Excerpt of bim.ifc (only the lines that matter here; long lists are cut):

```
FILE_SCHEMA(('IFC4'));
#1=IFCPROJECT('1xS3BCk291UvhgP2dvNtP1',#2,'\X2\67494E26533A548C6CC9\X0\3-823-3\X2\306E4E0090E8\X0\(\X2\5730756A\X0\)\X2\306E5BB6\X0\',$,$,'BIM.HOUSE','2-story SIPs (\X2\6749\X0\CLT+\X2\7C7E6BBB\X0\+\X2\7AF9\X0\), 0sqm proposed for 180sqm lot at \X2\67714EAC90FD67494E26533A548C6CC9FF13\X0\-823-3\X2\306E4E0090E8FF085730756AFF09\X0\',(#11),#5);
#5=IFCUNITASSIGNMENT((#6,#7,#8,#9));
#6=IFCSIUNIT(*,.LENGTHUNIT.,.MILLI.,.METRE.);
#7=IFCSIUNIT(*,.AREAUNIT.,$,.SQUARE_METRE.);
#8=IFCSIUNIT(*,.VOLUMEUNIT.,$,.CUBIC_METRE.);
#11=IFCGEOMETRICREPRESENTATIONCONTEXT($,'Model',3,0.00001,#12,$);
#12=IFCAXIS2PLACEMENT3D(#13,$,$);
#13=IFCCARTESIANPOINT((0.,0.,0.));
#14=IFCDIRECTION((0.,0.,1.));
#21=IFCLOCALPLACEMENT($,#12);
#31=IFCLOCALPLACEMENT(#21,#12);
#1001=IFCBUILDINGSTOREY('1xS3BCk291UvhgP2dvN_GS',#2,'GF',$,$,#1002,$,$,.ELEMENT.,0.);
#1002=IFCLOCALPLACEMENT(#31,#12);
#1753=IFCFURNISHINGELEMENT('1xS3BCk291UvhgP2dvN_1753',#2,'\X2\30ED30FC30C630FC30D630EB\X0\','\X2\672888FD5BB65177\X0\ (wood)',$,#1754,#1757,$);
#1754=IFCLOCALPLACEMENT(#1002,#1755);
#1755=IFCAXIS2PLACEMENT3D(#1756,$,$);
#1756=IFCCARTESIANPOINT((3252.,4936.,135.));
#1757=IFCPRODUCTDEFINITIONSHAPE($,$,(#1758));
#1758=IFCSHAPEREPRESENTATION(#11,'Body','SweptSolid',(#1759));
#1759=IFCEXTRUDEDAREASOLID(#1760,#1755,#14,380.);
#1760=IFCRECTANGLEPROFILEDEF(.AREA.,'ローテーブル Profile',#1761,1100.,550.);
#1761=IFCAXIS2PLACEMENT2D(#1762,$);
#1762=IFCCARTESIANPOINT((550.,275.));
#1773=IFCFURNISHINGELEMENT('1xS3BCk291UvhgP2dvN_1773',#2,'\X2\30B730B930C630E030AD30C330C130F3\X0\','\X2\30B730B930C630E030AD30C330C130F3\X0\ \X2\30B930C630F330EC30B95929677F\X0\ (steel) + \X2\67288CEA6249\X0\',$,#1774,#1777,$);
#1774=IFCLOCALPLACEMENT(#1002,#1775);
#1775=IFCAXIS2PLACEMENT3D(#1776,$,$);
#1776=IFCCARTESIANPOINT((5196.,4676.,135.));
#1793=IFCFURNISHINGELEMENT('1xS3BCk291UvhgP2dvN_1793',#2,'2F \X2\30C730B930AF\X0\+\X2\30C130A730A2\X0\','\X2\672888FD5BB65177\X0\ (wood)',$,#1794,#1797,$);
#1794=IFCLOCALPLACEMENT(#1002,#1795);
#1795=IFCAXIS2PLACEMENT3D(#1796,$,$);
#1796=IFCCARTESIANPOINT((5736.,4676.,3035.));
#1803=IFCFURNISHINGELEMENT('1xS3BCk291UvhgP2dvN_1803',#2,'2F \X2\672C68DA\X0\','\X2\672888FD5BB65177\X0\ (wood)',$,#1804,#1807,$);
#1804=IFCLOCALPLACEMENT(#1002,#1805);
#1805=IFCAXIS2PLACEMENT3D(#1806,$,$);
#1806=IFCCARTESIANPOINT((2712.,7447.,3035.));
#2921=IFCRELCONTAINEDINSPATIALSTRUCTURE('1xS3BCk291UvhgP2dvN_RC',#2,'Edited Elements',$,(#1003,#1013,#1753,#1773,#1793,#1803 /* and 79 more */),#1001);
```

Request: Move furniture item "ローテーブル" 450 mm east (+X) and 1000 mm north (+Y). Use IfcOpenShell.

```python
import ifcopenshell
import ifcopenshell.api.geometry
import ifcopenshell.util.placement
import ifcopenshell.util.unit

model = ifcopenshell.open("bim.ifc")
unit_scale = ifcopenshell.util.unit.calculate_unit_scale(model)

item = model.by_id(1753)
matrix = ifcopenshell.util.placement.get_local_placement(item.ObjectPlacement)
matrix[0, 3] += 0.45 / unit_scale
matrix[1, 3] += 1 / unit_scale
ifcopenshell.api.geometry.edit_object_placement(model, product=item, matrix=matrix, is_si=False)

print(ifcopenshell.util.placement.get_local_placement(item.ObjectPlacement).round(3) + 0.0)

model.write("bim_edited.ifc")
```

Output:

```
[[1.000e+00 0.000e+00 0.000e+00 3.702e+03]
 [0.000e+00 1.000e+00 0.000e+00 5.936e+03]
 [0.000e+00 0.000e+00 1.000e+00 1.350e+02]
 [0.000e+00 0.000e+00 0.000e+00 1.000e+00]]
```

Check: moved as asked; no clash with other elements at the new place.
